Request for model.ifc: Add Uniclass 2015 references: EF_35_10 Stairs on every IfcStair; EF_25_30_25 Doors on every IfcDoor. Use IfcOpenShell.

First a look at what the model holds.

```python
import ifcopenshell

model = ifcopenshell.open("model.ifc")
print(model.schema)
print("classifications:", [c.Name for c in model.by_type("IfcClassification")])
for ifc_class in ("IfcDoor", "IfcRoof", "IfcStair", "IfcWall", "IfcWindow"):
    print(ifc_class, len(model.by_type(ifc_class)))
```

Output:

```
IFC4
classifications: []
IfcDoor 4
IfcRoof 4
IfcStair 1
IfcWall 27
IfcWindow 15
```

```python
import ifcopenshell
import ifcopenshell.api.classification

model = ifcopenshell.open("model.ifc")

system = ifcopenshell.api.classification.add_classification(model, classification="Uniclass 2015")

codes = {
    "IfcStair": ("EF_35_10", "Stairs"),
    "IfcDoor": ("EF_25_30_25", "Doors"),
}
for ifc_class, (code, name) in codes.items():
    products = model.by_type(ifc_class)
    ifcopenshell.api.classification.add_reference(
        model, products=products, classification=system, identification=code, name=name
    )
    print(code, len(products))

model.write("model_edited.ifc")
```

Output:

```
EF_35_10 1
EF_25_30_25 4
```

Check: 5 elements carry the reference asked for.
